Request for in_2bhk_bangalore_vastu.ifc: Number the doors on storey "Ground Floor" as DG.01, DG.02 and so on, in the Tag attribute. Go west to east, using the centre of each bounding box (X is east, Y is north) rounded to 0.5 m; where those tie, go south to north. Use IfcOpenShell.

First a look at what the model holds.

```python
import ifcopenshell
import ifcopenshell.util.element
import ifcopenshell.util.placement

model = ifcopenshell.open("in_2bhk_bangalore_vastu.ifc")
print(model.schema)
storey = next(s for s in model.by_type("IfcBuildingStorey") if s.Name == "Ground Floor")
doors = [e for e in ifcopenshell.util.element.get_decomposition(storey) if e.is_a("IfcDoor")]
for e in sorted(doors, key=lambda e: e.id()):
    origin = ifcopenshell.util.placement.get_local_placement(e.ObjectPlacement)[:3, 3]
    print(e.id(), e.Tag, e.Name, origin.round(2) + 0.0, sep=" | ")
```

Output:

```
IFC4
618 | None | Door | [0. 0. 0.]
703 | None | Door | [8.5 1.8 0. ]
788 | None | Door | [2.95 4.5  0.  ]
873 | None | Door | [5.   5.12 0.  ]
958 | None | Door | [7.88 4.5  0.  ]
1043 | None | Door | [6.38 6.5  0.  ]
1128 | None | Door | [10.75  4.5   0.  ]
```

```python
import ifcopenshell
import ifcopenshell.geom
import ifcopenshell.util.element
import ifcopenshell.util.shape

model = ifcopenshell.open("in_2bhk_bangalore_vastu.ifc")
settings = ifcopenshell.geom.settings()
settings.set("use-world-coords", True)


def centre(element):
    shape = ifcopenshell.geom.create_shape(settings, element)
    return ifcopenshell.util.shape.get_bbox_centroid(shape.geometry)


storey = next(s for s in model.by_type("IfcBuildingStorey") if s.Name == "Ground Floor")
doors = [e for e in ifcopenshell.util.element.get_decomposition(storey) if e.is_a("IfcDoor")]

# Insertion points can sit at a corner or the storey origin, so sort by the geometry (in metres).
centres = {e: centre(e) for e in doors}
doors.sort(key=lambda e: (round(centres[e][0] / 0.5), centres[e][1]))

for i, e in enumerate(doors, start=1):
    number = f"DG.{i:02d}"
    e.Tag = number
    print(e.id(), number)

model.write("in_2bhk_bangalore_vastu-out.ifc")
```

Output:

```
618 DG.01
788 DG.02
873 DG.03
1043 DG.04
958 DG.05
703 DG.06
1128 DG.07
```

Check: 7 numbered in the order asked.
